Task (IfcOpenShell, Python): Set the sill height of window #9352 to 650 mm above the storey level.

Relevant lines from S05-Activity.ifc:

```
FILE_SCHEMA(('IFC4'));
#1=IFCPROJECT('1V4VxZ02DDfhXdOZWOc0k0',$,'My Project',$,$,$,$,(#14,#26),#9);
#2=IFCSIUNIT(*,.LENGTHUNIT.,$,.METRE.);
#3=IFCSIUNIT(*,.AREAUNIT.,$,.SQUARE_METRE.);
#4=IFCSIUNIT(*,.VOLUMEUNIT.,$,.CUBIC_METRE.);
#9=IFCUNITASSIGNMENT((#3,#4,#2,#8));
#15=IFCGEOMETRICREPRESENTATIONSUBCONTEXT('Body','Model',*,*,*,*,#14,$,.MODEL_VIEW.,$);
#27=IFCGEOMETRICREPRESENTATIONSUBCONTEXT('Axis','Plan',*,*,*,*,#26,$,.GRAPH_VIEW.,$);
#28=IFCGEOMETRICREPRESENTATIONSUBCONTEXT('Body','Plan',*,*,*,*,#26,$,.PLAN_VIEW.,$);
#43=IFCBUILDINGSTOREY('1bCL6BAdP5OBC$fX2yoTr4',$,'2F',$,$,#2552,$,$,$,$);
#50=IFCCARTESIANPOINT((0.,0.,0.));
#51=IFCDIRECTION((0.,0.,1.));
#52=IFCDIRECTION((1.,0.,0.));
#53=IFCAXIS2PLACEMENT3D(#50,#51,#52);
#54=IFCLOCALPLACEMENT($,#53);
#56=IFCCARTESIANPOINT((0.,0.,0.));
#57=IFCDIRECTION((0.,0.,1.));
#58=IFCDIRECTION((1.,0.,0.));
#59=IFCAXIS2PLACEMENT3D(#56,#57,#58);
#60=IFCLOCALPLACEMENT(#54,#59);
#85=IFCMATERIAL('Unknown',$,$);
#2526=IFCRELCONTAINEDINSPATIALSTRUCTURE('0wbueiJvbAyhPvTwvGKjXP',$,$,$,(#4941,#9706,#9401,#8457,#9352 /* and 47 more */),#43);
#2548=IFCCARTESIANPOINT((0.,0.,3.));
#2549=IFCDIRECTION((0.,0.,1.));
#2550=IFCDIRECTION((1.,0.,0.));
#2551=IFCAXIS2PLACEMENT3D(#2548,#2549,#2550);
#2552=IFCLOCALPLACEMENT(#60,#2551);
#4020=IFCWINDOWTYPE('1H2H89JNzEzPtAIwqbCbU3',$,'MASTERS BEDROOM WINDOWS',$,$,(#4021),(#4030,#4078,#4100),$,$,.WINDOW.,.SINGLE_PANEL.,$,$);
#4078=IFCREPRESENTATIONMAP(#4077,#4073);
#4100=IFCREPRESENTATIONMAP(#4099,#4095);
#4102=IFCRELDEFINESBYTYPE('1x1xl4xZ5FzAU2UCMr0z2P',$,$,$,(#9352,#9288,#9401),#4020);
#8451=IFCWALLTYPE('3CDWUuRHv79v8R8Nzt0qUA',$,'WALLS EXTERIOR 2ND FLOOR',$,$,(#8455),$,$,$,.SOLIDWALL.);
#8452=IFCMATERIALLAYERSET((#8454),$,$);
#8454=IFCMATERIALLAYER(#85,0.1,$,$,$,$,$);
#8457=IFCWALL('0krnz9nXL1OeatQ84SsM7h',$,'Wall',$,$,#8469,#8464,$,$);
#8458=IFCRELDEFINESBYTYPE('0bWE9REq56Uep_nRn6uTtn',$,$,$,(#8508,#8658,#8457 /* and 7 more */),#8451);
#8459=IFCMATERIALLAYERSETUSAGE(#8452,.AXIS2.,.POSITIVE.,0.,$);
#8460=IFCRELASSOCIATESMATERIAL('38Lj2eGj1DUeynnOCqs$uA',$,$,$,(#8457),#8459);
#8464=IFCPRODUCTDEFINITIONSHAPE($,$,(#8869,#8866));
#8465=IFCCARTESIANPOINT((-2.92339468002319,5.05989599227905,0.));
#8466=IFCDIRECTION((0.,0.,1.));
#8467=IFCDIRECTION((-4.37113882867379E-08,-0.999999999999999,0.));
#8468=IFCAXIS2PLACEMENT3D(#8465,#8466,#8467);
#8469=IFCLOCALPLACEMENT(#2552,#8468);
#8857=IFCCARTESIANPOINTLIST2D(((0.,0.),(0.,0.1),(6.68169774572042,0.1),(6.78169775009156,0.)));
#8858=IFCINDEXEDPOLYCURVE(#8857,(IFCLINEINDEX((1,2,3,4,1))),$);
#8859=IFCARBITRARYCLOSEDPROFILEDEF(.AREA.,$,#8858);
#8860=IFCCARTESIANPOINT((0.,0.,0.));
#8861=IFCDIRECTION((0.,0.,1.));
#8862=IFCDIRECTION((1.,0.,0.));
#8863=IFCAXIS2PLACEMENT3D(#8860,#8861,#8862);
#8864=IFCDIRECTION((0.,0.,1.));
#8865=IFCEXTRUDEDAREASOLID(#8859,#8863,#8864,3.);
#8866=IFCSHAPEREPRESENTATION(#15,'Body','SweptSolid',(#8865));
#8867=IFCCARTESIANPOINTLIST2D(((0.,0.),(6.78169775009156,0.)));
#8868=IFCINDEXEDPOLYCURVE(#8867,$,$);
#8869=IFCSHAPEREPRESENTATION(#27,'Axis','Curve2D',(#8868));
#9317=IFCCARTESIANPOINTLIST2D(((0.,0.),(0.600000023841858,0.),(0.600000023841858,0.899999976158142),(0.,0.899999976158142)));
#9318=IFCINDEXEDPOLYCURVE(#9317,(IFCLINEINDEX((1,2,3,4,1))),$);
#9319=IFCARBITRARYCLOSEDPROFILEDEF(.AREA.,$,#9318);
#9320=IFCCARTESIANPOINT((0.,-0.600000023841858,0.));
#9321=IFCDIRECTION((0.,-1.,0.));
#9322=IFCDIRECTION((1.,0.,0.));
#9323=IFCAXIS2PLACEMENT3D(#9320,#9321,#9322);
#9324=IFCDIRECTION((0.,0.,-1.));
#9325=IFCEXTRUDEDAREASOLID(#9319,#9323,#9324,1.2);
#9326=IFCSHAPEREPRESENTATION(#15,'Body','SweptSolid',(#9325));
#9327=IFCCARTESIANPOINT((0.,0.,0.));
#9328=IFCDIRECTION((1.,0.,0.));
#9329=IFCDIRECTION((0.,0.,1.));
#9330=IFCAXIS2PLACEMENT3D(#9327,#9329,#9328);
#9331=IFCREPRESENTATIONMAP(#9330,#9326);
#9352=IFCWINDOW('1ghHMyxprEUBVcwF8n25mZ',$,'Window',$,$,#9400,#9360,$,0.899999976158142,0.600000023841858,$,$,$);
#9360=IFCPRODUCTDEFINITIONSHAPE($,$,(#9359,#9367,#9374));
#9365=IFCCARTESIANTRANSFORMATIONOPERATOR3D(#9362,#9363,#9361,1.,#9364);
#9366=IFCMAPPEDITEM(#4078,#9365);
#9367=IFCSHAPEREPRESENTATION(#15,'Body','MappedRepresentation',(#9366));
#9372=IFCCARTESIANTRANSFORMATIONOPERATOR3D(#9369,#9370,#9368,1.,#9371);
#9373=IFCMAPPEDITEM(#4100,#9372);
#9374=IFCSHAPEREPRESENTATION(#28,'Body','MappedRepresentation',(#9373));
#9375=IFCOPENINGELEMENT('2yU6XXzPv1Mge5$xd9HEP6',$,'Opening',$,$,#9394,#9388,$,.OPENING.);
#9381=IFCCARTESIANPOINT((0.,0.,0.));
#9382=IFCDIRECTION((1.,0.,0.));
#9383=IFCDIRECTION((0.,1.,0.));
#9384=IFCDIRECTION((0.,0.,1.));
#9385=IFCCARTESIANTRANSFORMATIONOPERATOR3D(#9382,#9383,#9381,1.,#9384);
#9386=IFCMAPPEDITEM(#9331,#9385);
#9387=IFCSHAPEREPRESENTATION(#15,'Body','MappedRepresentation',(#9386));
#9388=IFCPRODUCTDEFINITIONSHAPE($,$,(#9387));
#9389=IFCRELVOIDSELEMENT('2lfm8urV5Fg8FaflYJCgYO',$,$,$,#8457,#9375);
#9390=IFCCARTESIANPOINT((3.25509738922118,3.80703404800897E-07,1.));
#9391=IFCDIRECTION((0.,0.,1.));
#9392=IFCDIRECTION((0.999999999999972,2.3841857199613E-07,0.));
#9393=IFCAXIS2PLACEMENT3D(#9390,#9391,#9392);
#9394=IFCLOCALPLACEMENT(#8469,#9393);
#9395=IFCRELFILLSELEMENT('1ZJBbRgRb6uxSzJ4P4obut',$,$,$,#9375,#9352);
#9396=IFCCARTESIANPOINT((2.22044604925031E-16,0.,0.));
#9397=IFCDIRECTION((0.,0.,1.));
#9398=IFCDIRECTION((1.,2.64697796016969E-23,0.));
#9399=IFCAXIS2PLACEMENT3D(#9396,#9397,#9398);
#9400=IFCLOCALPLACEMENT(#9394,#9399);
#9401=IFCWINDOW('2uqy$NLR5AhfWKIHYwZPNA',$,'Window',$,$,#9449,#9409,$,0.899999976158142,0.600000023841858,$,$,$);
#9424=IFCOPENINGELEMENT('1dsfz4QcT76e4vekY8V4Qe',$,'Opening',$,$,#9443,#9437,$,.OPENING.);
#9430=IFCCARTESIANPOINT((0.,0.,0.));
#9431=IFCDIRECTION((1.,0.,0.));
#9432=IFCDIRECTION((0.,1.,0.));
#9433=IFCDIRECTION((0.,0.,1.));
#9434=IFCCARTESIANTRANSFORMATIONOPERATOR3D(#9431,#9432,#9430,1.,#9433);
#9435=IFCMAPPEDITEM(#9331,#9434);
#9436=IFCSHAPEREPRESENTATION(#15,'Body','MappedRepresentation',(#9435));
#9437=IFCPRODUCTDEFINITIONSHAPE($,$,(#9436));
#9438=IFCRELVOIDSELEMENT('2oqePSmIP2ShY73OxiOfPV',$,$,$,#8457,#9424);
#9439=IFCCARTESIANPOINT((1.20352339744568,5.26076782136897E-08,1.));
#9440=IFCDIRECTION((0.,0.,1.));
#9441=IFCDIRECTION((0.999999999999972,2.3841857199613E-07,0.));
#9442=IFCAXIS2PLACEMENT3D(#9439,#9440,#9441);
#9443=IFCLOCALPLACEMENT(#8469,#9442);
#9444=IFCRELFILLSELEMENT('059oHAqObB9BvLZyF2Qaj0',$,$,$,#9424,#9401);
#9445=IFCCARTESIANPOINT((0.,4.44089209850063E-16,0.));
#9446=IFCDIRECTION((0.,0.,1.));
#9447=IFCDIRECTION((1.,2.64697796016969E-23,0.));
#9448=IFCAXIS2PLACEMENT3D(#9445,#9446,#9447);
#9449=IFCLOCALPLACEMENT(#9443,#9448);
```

```python
import numpy as np
import ifcopenshell
import ifcopenshell.api.geometry
import ifcopenshell.geom
import ifcopenshell.util.element
import ifcopenshell.util.placement
import ifcopenshell.util.shape
import ifcopenshell.util.unit

model = ifcopenshell.open("S05-Activity.ifc")
unit_scale = ifcopenshell.util.unit.calculate_unit_scale(model)

window = model.by_guid("1ghHMyxprEUBVcwF8n25mZ")
opening = window.FillsVoids[0].RelatingOpeningElement
storey = ifcopenshell.util.element.get_container(window, ifc_class="IfcBuildingStorey")
level = ifcopenshell.util.placement.get_local_placement(storey.ObjectPlacement)[2, 3]

# The opening's origin need not be at the sill, so measure its lowest point.
shape = ifcopenshell.geom.create_shape(ifcopenshell.geom.settings(), opening)
bottom = ifcopenshell.util.shape.get_shape_bottom_elevation(shape, shape.geometry) / unit_scale
dz = level + 0.65 - bottom

shift = np.array([0.0, 0.0, dz])
# The window is placed relative to its opening, so it follows when the opening moves.
matrix = ifcopenshell.util.placement.get_local_placement(opening.ObjectPlacement)
matrix[:3, 3] += shift
ifcopenshell.api.geometry.edit_object_placement(
    model, product=opening, matrix=matrix, is_si=False, should_transform_children=True
)

print(f"moved by {dz * unit_scale:+.3f} m")

model.write("S05-Activity_rev.ifc")
```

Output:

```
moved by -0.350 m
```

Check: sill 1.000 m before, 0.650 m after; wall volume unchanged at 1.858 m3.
